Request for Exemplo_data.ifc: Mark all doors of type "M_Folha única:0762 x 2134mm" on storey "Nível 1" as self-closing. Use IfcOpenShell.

First a look at what the model holds.

```python
import ifcopenshell
import ifcopenshell.util.element

model = ifcopenshell.open("Exemplo_data.ifc")
print(model.schema)
storey = next(s for s in model.by_type("IfcBuildingStorey") if s.Name == "Nível 1")
doors = [e for e in ifcopenshell.util.element.get_decomposition(storey) if e.is_a("IfcDoor")]
seen = {}
for e in doors:
    element_type = ifcopenshell.util.element.get_type(e)
    key = (element_type.Name if element_type != e and element_type else None, ifcopenshell.util.element.get_pset(e, "Pset_DoorCommon", "SelfClosing"))
    seen[key] = seen.get(key, 0) + 1
for (name, value), count in sorted(seen.items(), key=str):
    print(count, "x", name, "|", value)
```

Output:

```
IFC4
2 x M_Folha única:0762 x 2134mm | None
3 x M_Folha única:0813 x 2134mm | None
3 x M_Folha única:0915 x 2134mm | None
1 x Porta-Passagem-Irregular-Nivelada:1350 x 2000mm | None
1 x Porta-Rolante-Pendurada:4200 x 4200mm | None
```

```python
import ifcopenshell
import ifcopenshell.api.pset
import ifcopenshell.util.element

model = ifcopenshell.open("Exemplo_data.ifc")

storey = next(s for s in model.by_type("IfcBuildingStorey") if s.Name == "Nível 1")
doors = [e for e in ifcopenshell.util.element.get_decomposition(storey) if e.is_a("IfcDoor")]

count = 0
for e in doors:
    element_type = ifcopenshell.util.element.get_type(e)
    if element_type in (None, e) or element_type.Name != "M_Folha única:0762 x 2134mm":
        continue
    # add_pset returns the element's existing set when there is one.
    pset = ifcopenshell.api.pset.add_pset(model, product=e, name="Pset_DoorCommon")
    ifcopenshell.api.pset.edit_pset(model, pset=pset, properties={"SelfClosing": True})
    count += 1

print(count, "doors updated")

model.write("Exemplo_data_updated.ifc")
```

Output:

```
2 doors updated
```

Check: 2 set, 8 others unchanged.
